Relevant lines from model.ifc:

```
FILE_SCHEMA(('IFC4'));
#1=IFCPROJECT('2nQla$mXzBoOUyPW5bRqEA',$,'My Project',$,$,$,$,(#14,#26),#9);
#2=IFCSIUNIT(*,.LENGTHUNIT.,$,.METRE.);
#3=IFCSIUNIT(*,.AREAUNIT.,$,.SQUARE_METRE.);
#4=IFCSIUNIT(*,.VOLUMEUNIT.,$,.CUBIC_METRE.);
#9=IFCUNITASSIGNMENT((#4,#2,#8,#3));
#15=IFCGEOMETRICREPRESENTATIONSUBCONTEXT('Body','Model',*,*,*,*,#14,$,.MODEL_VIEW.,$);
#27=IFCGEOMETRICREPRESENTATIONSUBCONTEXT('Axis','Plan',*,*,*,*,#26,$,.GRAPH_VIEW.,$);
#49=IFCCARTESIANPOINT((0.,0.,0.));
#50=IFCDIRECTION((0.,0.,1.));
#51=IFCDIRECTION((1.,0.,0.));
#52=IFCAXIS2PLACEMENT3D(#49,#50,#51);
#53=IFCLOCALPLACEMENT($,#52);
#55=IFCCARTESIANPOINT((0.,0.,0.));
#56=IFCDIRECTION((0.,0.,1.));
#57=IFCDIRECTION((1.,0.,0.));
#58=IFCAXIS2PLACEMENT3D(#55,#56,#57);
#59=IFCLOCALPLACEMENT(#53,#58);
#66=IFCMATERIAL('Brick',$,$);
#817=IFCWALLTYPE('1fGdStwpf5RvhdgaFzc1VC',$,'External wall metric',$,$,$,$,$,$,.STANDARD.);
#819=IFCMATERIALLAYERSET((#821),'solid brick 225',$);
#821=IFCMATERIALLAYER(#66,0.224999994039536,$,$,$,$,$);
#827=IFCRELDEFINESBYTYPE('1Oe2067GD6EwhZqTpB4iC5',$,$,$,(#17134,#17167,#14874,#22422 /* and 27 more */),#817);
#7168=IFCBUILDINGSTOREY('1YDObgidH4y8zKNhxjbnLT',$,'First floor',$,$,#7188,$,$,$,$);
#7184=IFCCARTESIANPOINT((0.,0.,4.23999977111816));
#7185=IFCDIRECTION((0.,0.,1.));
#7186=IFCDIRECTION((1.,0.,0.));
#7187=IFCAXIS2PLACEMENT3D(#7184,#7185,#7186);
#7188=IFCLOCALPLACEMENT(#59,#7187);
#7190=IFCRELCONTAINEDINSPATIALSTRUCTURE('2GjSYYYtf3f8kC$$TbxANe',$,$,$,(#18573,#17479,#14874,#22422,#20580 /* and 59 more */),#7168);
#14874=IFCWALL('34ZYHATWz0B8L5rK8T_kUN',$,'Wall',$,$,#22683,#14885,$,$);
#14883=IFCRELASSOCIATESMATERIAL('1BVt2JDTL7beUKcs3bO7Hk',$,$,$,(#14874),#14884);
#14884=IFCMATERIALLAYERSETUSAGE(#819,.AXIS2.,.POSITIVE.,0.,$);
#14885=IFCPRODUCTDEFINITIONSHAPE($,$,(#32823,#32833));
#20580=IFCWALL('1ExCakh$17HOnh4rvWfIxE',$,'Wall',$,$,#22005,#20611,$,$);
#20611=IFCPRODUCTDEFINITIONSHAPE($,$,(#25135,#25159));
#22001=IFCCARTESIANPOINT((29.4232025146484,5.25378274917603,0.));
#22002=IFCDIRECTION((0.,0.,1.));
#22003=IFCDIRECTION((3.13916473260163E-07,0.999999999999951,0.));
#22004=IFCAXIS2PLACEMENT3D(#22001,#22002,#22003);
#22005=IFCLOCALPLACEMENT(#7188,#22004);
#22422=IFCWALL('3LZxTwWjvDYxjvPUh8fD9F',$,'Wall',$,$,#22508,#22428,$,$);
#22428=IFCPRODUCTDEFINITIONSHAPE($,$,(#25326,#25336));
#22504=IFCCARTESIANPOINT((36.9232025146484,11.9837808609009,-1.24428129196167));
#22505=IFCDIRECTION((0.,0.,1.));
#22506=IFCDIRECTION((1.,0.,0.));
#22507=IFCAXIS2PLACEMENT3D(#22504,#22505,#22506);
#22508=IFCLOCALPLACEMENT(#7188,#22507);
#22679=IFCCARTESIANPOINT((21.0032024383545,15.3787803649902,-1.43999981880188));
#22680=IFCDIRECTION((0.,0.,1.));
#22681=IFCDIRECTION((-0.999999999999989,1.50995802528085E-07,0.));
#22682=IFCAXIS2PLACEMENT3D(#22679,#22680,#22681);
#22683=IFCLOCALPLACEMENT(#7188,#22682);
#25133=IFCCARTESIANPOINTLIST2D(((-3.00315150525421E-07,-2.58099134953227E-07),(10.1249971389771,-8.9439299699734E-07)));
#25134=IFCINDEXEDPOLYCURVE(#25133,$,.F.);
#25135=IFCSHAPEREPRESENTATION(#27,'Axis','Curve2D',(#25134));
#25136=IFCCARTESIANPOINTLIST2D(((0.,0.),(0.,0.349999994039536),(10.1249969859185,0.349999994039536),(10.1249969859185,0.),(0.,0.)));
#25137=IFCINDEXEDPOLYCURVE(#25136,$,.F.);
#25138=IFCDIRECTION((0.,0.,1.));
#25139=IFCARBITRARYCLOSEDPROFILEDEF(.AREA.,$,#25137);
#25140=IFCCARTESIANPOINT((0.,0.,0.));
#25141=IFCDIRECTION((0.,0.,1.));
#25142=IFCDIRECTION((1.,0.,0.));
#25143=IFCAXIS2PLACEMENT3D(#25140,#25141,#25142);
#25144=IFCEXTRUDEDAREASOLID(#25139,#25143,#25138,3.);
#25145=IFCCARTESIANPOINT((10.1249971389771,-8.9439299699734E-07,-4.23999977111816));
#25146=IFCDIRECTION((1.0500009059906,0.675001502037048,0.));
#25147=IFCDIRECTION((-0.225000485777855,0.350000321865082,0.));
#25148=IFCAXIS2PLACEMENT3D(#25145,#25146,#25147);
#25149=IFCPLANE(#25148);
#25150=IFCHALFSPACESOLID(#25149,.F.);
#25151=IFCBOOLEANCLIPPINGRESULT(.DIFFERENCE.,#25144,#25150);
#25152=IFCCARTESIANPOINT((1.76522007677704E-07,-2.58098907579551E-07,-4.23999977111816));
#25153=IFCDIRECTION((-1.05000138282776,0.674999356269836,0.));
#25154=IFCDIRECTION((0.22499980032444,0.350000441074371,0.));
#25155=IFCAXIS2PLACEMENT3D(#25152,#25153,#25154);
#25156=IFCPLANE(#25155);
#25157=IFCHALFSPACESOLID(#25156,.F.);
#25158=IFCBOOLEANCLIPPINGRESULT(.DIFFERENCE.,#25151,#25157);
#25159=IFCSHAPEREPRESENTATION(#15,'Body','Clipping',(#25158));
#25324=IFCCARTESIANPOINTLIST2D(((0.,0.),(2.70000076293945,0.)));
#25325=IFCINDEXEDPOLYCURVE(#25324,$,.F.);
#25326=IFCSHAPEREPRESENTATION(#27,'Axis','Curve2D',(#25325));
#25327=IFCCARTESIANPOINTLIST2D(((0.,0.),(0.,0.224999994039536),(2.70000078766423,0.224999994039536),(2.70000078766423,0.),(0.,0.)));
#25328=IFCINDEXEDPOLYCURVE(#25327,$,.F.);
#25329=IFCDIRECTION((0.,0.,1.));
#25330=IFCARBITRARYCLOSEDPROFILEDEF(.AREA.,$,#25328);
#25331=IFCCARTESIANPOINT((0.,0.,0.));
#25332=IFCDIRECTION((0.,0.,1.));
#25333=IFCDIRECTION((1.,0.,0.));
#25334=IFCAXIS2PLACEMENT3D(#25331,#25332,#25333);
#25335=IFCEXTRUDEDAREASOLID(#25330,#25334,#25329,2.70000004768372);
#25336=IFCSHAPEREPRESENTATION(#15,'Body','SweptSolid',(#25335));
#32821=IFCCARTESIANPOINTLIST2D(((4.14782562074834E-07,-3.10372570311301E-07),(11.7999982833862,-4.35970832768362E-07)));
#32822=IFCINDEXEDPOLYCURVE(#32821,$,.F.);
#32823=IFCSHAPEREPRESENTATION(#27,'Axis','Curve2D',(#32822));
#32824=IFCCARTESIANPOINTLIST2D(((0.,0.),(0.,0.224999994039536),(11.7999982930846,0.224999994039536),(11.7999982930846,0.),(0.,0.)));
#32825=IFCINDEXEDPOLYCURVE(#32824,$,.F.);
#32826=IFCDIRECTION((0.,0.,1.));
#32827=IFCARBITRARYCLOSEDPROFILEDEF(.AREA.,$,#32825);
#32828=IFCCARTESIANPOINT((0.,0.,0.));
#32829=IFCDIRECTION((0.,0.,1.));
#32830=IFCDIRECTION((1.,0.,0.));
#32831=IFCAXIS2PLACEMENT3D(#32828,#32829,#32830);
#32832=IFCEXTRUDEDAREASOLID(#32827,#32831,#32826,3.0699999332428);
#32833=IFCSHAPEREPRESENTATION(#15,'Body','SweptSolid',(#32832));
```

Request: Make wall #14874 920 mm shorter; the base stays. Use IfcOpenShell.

```python
import ifcopenshell
import ifcopenshell.geom
import ifcopenshell.util.representation
import ifcopenshell.util.shape

model = ifcopenshell.open("model.ifc")
settings = ifcopenshell.geom.settings()


def volume(element):
    """Net volume in cubic metres, openings subtracted."""
    shape = ifcopenshell.geom.create_shape(settings, element)
    return ifcopenshell.util.shape.get_volume(shape.geometry)


wall = model.by_guid("34ZYHATWz0B8L5rK8T_kUN")
before = volume(wall)

body = ifcopenshell.util.representation.get_representation(wall, "Model", "Body")
solid = body.Items[0]
old_height = solid.Depth
solid.Depth -= 0.92
after = volume(wall)

print(f"height {old_height:g} -> {solid.Depth:g}, volume {before:.3f} -> {after:.3f} m3")

model.write("model_v2.ifc")
```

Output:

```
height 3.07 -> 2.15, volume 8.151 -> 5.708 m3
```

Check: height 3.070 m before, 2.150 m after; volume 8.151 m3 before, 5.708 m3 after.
